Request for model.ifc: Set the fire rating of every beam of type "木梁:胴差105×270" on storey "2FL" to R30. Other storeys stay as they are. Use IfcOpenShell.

First a look at what the model holds.

```python
import ifcopenshell
import ifcopenshell.util.element

model = ifcopenshell.open("model.ifc")
print(model.schema)
storey = next(s for s in model.by_type("IfcBuildingStorey") if s.Name == "2FL")
beams = [e for e in ifcopenshell.util.element.get_decomposition(storey) if e.is_a("IfcBeam")]
seen = {}
for e in beams:
    element_type = ifcopenshell.util.element.get_type(e)
    key = (element_type.Name if element_type != e and element_type else None, ifcopenshell.util.element.get_pset(e, "Pset_BeamCommon", "FireRating"))
    seen[key] = seen.get(key, 0) + 1
for (name, value), count in sorted(seen.items(), key=str):
    print(count, "x", name, "|", value)
```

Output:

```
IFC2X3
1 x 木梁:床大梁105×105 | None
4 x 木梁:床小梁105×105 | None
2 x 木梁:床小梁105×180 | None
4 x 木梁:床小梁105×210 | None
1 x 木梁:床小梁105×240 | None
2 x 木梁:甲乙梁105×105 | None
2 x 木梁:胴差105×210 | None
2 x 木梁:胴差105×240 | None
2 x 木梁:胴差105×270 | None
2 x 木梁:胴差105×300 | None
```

```python
import ifcopenshell
import ifcopenshell.api.pset
import ifcopenshell.util.element

model = ifcopenshell.open("model.ifc")

storey = next(s for s in model.by_type("IfcBuildingStorey") if s.Name == "2FL")
beams = [e for e in ifcopenshell.util.element.get_decomposition(storey) if e.is_a("IfcBeam")]

count = 0
for e in beams:
    element_type = ifcopenshell.util.element.get_type(e)
    if element_type in (None, e) or element_type.Name != "木梁:胴差105×270":
        continue
    # add_pset returns the element's existing set when there is one.
    pset = ifcopenshell.api.pset.add_pset(model, product=e, name="Pset_BeamCommon")
    ifcopenshell.api.pset.edit_pset(model, pset=pset, properties={"FireRating": "R30"})
    count += 1

print(count, "beams updated")

model.write("model_edited.ifc")
```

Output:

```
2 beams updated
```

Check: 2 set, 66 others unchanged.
